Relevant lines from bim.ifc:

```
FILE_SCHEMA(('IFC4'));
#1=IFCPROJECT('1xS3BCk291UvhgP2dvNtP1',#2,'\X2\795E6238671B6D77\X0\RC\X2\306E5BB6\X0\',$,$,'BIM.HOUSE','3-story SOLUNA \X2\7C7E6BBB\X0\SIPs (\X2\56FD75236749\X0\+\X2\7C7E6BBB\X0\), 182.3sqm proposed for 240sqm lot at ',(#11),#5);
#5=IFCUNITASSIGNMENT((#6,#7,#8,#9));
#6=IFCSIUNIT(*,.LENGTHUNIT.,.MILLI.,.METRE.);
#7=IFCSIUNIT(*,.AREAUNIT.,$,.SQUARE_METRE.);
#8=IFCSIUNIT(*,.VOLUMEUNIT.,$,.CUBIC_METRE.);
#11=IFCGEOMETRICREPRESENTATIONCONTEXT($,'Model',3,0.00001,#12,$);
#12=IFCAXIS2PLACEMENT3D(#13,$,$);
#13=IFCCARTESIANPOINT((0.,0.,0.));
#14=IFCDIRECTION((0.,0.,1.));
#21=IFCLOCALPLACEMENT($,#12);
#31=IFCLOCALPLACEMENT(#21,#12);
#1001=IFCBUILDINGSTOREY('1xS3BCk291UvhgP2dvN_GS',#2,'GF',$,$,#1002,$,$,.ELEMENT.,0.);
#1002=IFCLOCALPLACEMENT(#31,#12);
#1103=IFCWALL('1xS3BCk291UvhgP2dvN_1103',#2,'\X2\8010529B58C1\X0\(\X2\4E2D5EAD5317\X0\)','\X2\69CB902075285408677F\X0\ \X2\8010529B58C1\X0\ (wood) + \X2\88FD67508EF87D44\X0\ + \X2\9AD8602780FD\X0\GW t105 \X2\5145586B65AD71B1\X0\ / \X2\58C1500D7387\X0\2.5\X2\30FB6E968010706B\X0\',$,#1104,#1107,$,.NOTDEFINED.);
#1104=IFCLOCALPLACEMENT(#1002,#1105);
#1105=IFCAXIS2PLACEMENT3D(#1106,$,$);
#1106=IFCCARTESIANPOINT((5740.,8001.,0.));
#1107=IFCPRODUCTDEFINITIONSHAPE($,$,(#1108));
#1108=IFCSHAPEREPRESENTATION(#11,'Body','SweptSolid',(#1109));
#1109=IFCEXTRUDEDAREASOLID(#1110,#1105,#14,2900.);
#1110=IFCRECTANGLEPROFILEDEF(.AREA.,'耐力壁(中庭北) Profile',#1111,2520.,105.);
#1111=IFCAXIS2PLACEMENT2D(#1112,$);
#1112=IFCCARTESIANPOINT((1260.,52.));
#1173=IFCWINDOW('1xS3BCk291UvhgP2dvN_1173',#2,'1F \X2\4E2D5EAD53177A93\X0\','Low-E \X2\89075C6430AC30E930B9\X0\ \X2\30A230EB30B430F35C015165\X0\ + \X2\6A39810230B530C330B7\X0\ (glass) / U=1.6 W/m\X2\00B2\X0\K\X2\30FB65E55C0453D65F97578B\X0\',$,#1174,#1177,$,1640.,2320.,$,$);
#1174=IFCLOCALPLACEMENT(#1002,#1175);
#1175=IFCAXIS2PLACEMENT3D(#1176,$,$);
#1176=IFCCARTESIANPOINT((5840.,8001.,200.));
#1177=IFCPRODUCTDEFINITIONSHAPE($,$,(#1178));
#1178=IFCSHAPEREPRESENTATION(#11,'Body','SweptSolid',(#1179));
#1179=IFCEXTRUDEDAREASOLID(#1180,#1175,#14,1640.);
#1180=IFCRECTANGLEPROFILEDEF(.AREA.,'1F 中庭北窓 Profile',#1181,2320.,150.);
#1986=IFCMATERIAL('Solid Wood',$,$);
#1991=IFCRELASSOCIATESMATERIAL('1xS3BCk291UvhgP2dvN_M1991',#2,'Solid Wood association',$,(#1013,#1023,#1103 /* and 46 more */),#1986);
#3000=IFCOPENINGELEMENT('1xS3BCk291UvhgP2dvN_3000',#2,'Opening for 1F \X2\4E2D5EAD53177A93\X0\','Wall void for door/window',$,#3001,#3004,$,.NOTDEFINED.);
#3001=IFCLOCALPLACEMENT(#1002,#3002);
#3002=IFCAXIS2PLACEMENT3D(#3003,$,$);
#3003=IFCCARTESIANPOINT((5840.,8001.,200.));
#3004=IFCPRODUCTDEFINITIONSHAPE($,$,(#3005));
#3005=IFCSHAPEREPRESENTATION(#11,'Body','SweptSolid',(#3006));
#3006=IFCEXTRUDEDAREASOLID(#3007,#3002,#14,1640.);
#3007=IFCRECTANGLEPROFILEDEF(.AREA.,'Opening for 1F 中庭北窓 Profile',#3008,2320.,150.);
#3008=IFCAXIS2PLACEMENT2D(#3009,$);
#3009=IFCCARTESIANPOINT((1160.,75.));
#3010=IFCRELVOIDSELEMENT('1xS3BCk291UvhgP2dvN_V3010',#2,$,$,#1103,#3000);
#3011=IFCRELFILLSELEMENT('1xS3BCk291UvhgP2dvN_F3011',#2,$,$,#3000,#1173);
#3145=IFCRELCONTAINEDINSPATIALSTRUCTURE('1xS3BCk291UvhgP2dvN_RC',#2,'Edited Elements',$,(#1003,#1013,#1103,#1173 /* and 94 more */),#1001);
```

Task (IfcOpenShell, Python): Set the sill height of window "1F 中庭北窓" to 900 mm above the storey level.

```python
import numpy as np
import ifcopenshell
import ifcopenshell.api.geometry
import ifcopenshell.geom
import ifcopenshell.util.element
import ifcopenshell.util.placement
import ifcopenshell.util.shape
import ifcopenshell.util.unit

model = ifcopenshell.open("bim.ifc")
unit_scale = ifcopenshell.util.unit.calculate_unit_scale(model)

window = model.by_guid("1xS3BCk291UvhgP2dvN_1173")
opening = window.FillsVoids[0].RelatingOpeningElement
storey = ifcopenshell.util.element.get_container(window, ifc_class="IfcBuildingStorey")
level = ifcopenshell.util.placement.get_local_placement(storey.ObjectPlacement)[2, 3]

# The opening's origin need not be at the sill, so measure its lowest point.
shape = ifcopenshell.geom.create_shape(ifcopenshell.geom.settings(), opening)
bottom = ifcopenshell.util.shape.get_shape_bottom_elevation(shape, shape.geometry) / unit_scale
dz = level + 0.9 / unit_scale - bottom

shift = np.array([0.0, 0.0, dz])
# The window is not placed relative to its opening, so move both.
for product in (opening, window):
    matrix = ifcopenshell.util.placement.get_local_placement(product.ObjectPlacement)
    matrix[:3, 3] += shift
    ifcopenshell.api.geometry.edit_object_placement(model, product=product, matrix=matrix, is_si=False)

print(f"moved by {dz * unit_scale:+.3f} m")

model.write("bim-out.ifc")
```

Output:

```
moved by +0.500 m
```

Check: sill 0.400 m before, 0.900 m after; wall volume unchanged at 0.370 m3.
